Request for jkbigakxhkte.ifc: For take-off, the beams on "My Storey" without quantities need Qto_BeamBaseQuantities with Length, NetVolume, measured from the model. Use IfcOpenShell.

First a look at what the model holds.

```python
import ifcopenshell
import ifcopenshell.util.element
import ifcopenshell.util.unit

model = ifcopenshell.open("jkbigakxhkte.ifc")
print(model.schema)
for unit_type in ("LENGTHUNIT", "AREAUNIT", "VOLUMEUNIT"):
    print(unit_type, ifcopenshell.util.unit.calculate_unit_scale(model, unit_type))
storey = next(s for s in model.by_type("IfcBuildingStorey") if s.Name == "My Storey")
beams = [e for e in ifcopenshell.util.element.get_decomposition(storey) if e.is_a("IfcBeam")]
for e in sorted(beams, key=lambda e: e.id()):
    print(e.id(), e.is_a(), e.Name, list(ifcopenshell.util.element.get_psets(e, qtos_only=True)), sep=" | ")
```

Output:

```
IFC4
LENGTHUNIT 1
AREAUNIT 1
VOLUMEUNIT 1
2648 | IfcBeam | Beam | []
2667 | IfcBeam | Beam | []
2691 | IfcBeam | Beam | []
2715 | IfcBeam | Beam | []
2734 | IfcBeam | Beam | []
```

```python
import ifcopenshell
import ifcopenshell.api.pset
import ifcopenshell.geom
import ifcopenshell.util.element
import ifcopenshell.util.shape
import ifcopenshell.util.unit

model = ifcopenshell.open("jkbigakxhkte.ifc")
unit_scale = ifcopenshell.util.unit.calculate_unit_scale(model)
volume_scale = ifcopenshell.util.unit.calculate_unit_scale(model, "VOLUMEUNIT")
settings = ifcopenshell.geom.settings()

storey = next(s for s in model.by_type("IfcBuildingStorey") if s.Name == "My Storey")
beams = [e for e in ifcopenshell.util.element.get_decomposition(storey) if e.is_a("IfcBeam")]

for e in sorted(beams, key=lambda e: e.id()):
    if ifcopenshell.util.element.get_psets(e, qtos_only=True, should_inherit=False):
        continue
    # Geometry comes back in metres, in the element's own axes.
    shape = ifcopenshell.geom.create_shape(settings, e)
    values = {
        "Length": ifcopenshell.util.shape.get_max_xyz(shape.geometry) / unit_scale,
        "NetVolume": ifcopenshell.util.shape.get_volume(shape.geometry) / volume_scale,
    }
    qto = ifcopenshell.api.pset.add_qto(model, product=e, name="Qto_BeamBaseQuantities")
    ifcopenshell.api.pset.edit_qto(model, qto=qto, properties=values)
    print(e.id(), {k: round(v, 3) for k, v in values.items()})

model.write("jkbigakxhkte_rev.ifc")
```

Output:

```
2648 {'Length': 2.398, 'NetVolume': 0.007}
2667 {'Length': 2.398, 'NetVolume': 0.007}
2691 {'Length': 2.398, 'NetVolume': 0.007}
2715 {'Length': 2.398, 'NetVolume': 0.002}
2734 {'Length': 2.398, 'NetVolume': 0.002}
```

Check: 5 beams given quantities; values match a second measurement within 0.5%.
